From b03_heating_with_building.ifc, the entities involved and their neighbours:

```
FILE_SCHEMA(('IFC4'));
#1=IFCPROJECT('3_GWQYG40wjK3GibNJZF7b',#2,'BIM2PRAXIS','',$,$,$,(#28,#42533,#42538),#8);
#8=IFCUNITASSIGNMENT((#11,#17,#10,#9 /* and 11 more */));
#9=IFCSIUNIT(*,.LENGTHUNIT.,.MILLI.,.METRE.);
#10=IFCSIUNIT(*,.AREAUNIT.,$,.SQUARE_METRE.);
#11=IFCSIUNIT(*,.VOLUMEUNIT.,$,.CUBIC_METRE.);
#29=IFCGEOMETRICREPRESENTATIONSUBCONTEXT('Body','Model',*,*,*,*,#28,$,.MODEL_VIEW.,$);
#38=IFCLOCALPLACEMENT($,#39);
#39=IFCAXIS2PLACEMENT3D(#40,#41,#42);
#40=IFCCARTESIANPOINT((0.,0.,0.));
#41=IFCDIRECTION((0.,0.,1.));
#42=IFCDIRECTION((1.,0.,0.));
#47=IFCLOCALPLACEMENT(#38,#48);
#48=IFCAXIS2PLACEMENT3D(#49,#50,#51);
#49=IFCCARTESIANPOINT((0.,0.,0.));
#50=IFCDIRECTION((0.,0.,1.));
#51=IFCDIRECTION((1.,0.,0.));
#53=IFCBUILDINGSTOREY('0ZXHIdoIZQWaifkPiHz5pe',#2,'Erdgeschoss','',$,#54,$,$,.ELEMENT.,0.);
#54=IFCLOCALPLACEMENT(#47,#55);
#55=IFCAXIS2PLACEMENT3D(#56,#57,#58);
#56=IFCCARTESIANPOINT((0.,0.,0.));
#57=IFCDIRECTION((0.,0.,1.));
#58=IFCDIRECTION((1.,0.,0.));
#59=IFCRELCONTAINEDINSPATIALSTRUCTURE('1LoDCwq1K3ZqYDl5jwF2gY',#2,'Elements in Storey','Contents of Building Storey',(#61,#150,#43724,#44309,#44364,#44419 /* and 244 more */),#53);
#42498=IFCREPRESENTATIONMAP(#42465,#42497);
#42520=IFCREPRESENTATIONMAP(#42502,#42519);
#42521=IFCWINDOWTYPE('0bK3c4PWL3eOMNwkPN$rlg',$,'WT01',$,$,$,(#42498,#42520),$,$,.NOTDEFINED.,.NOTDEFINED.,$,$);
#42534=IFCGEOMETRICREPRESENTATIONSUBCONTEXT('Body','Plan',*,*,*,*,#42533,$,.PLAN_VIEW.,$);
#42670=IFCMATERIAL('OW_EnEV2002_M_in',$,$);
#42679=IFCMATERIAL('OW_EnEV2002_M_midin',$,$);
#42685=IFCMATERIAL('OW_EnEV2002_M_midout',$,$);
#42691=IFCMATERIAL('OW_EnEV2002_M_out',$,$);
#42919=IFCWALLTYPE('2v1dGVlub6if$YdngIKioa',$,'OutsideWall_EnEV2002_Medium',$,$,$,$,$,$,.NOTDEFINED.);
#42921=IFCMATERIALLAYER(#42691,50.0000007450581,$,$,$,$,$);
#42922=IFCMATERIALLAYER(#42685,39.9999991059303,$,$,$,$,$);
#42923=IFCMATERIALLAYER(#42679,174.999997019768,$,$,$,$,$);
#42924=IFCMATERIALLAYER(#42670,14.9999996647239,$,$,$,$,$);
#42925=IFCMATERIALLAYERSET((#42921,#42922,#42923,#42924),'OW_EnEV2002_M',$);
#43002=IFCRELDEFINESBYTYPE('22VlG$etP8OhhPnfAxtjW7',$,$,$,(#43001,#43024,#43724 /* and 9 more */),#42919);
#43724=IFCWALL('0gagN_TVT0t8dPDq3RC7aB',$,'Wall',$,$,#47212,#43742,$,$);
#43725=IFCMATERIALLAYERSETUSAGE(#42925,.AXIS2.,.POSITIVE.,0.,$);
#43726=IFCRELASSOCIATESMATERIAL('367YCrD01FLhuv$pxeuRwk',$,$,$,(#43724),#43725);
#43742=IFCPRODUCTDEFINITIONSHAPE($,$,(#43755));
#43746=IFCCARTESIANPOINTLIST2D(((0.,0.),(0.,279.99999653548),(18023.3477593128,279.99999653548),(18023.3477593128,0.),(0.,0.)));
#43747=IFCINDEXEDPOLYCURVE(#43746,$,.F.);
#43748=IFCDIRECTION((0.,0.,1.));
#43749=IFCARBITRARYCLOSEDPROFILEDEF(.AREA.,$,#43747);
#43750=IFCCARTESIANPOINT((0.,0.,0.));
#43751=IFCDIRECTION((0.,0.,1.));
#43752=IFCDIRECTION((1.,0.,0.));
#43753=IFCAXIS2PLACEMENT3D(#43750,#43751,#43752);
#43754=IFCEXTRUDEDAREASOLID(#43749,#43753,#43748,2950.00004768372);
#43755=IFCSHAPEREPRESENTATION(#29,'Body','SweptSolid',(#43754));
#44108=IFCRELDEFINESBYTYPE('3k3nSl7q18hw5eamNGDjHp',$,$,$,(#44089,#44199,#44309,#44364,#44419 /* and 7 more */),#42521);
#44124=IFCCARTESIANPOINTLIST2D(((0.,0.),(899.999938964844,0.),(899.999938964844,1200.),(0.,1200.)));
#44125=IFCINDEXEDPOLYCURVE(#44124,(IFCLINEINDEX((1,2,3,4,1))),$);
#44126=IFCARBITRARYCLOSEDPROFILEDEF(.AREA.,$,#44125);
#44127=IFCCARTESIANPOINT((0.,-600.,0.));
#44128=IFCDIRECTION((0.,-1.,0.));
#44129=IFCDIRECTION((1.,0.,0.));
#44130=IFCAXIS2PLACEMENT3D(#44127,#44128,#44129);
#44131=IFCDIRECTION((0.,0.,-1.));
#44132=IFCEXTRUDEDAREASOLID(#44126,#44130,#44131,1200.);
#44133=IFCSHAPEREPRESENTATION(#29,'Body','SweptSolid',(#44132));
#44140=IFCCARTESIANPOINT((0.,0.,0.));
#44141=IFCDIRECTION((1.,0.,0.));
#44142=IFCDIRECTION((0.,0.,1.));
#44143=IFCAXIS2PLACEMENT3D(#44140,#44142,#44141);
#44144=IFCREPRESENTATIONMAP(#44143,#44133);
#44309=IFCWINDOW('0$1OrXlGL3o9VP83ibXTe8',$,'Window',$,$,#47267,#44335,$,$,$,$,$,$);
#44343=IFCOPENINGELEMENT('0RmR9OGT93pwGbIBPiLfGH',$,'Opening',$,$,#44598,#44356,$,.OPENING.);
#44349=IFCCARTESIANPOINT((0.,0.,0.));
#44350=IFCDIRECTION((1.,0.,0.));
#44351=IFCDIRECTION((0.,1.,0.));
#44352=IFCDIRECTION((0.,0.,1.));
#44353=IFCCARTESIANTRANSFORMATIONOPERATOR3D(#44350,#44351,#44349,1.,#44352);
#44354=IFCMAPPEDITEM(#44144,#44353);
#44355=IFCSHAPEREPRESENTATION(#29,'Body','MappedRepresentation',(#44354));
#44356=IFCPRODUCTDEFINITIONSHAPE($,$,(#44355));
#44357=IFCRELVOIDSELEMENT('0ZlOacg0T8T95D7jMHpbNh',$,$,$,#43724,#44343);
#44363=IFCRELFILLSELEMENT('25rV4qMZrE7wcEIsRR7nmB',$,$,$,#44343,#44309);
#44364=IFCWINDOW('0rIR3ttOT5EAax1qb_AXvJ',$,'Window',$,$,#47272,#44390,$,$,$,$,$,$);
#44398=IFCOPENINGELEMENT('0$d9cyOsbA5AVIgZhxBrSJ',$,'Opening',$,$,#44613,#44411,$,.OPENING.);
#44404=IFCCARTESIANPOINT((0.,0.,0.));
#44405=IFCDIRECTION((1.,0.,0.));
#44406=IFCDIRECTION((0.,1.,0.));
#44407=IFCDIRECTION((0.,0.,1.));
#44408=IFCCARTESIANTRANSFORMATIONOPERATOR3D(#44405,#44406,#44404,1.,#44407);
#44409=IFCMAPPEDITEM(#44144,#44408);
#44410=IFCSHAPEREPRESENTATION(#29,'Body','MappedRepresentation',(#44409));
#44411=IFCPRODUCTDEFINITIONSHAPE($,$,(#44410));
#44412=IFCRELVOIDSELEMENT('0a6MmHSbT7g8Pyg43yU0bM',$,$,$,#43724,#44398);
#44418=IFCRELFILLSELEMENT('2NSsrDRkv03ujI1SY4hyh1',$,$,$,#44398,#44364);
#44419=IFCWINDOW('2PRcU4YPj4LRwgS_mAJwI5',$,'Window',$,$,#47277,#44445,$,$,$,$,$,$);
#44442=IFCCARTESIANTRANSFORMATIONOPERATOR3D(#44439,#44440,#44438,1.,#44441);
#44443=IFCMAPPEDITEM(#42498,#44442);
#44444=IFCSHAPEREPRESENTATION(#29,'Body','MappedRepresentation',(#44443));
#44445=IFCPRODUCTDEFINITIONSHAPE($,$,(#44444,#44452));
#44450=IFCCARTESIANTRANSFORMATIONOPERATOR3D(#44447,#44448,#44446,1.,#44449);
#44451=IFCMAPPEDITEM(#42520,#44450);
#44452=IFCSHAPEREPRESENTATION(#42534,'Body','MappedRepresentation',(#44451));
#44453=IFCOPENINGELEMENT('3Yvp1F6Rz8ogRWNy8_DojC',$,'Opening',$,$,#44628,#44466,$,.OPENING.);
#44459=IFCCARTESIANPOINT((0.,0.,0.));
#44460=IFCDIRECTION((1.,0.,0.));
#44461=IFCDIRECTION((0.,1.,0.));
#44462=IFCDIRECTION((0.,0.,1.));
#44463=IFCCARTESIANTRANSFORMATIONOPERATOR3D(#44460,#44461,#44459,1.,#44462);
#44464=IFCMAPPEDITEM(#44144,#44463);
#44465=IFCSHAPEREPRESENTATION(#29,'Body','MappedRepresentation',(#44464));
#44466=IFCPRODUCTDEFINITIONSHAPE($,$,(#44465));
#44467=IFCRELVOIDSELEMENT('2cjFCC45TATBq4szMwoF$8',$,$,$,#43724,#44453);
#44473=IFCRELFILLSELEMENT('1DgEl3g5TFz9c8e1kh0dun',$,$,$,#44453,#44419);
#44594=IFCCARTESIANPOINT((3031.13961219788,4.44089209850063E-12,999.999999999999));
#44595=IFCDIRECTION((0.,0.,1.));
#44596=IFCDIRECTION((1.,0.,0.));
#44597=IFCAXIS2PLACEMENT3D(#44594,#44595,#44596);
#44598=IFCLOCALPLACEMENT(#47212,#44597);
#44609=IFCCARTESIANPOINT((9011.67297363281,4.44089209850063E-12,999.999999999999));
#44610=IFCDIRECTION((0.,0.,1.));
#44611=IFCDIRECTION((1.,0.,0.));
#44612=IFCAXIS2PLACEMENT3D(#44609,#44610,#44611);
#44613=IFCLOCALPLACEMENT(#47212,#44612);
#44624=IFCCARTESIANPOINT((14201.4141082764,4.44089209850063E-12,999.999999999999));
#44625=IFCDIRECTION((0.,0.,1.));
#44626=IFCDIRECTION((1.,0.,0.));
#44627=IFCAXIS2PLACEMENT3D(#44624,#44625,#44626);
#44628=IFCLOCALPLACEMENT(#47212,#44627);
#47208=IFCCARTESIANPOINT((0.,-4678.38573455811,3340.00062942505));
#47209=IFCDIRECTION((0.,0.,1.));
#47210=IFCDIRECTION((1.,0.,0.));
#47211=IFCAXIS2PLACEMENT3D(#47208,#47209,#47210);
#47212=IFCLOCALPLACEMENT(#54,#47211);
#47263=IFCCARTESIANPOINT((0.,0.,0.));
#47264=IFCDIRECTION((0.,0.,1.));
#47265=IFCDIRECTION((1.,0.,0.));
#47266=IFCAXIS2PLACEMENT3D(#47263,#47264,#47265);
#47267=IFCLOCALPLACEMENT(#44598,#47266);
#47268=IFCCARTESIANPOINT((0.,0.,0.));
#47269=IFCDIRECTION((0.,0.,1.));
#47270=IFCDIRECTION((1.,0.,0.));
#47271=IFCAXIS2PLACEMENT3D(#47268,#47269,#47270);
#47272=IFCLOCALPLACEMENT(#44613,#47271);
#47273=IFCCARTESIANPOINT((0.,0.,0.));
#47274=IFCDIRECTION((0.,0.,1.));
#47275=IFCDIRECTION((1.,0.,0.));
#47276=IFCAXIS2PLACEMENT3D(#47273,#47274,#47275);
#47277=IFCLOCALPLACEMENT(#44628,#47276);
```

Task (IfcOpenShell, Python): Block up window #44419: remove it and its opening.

```python
import ifcopenshell
import ifcopenshell.api.feature
import ifcopenshell.api.root
import ifcopenshell.geom
import ifcopenshell.util.shape

model = ifcopenshell.open("b03_heating_with_building.ifc")
settings = ifcopenshell.geom.settings()


def volume(element):
    """Net volume in cubic metres, openings subtracted."""
    shape = ifcopenshell.geom.create_shape(settings, element)
    return ifcopenshell.util.shape.get_volume(shape.geometry)


window = model.by_id(44419)
opening = window.FillsVoids[0].RelatingOpeningElement
wall = opening.VoidsElements[0].RelatingBuildingElement
before = volume(wall)

ifcopenshell.api.root.remove_product(model, product=window)
ifcopenshell.api.feature.remove_feature(model, feature=opening)

after = volume(wall)

print(f"wall volume {before:.3f} -> {after:.3f} m3")

model.write("b03_heating_with_building_edited.ifc")
```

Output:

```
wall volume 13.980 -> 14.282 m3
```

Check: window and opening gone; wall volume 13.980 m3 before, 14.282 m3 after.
